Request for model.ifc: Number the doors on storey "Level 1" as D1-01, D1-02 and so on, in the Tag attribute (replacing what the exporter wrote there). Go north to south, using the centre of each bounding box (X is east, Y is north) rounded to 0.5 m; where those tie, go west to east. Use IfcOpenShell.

First a look at what the model holds.

```python
import ifcopenshell
import ifcopenshell.util.element
import ifcopenshell.util.placement

model = ifcopenshell.open("model.ifc")
print(model.schema)
storey = next(s for s in model.by_type("IfcBuildingStorey") if s.Name == "Level 1")
doors = [e for e in ifcopenshell.util.element.get_decomposition(storey) if e.is_a("IfcDoor")]
for e in sorted(doors, key=lambda e: e.id()):
    origin = ifcopenshell.util.placement.get_local_placement(e.ObjectPlacement)[:3, 3]
    print(e.id(), e.Tag, e.Name, origin.round(2) + 0.0, sep=" | ")
```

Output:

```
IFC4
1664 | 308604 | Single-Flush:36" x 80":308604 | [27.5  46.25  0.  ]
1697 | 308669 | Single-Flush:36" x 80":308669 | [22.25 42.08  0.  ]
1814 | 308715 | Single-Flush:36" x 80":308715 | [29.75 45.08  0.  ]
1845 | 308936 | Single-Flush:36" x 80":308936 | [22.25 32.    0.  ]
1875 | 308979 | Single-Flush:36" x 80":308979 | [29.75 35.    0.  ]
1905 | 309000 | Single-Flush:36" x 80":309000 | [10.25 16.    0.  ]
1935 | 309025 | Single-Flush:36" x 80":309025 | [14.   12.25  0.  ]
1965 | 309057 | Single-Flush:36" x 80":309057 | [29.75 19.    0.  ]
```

```python
import ifcopenshell
import ifcopenshell.geom
import ifcopenshell.util.element
import ifcopenshell.util.shape

model = ifcopenshell.open("model.ifc")
settings = ifcopenshell.geom.settings()
settings.set("use-world-coords", True)


def centre(element):
    shape = ifcopenshell.geom.create_shape(settings, element)
    return ifcopenshell.util.shape.get_bbox_centroid(shape.geometry)


storey = next(s for s in model.by_type("IfcBuildingStorey") if s.Name == "Level 1")
doors = [e for e in ifcopenshell.util.element.get_decomposition(storey) if e.is_a("IfcDoor")]

# Insertion points can sit at a corner or the storey origin, so sort by the geometry (in metres).
centres = {e: centre(e) for e in doors}
doors.sort(key=lambda e: (-round(centres[e][1] / 0.5), centres[e][0]))

for i, e in enumerate(doors, start=1):
    number = f"D1-{i:02d}"
    e.Tag = number
    print(e.id(), number)

model.write("model_rev.ifc")
```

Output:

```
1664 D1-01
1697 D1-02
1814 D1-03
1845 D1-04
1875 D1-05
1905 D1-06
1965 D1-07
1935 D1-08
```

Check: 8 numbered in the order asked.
